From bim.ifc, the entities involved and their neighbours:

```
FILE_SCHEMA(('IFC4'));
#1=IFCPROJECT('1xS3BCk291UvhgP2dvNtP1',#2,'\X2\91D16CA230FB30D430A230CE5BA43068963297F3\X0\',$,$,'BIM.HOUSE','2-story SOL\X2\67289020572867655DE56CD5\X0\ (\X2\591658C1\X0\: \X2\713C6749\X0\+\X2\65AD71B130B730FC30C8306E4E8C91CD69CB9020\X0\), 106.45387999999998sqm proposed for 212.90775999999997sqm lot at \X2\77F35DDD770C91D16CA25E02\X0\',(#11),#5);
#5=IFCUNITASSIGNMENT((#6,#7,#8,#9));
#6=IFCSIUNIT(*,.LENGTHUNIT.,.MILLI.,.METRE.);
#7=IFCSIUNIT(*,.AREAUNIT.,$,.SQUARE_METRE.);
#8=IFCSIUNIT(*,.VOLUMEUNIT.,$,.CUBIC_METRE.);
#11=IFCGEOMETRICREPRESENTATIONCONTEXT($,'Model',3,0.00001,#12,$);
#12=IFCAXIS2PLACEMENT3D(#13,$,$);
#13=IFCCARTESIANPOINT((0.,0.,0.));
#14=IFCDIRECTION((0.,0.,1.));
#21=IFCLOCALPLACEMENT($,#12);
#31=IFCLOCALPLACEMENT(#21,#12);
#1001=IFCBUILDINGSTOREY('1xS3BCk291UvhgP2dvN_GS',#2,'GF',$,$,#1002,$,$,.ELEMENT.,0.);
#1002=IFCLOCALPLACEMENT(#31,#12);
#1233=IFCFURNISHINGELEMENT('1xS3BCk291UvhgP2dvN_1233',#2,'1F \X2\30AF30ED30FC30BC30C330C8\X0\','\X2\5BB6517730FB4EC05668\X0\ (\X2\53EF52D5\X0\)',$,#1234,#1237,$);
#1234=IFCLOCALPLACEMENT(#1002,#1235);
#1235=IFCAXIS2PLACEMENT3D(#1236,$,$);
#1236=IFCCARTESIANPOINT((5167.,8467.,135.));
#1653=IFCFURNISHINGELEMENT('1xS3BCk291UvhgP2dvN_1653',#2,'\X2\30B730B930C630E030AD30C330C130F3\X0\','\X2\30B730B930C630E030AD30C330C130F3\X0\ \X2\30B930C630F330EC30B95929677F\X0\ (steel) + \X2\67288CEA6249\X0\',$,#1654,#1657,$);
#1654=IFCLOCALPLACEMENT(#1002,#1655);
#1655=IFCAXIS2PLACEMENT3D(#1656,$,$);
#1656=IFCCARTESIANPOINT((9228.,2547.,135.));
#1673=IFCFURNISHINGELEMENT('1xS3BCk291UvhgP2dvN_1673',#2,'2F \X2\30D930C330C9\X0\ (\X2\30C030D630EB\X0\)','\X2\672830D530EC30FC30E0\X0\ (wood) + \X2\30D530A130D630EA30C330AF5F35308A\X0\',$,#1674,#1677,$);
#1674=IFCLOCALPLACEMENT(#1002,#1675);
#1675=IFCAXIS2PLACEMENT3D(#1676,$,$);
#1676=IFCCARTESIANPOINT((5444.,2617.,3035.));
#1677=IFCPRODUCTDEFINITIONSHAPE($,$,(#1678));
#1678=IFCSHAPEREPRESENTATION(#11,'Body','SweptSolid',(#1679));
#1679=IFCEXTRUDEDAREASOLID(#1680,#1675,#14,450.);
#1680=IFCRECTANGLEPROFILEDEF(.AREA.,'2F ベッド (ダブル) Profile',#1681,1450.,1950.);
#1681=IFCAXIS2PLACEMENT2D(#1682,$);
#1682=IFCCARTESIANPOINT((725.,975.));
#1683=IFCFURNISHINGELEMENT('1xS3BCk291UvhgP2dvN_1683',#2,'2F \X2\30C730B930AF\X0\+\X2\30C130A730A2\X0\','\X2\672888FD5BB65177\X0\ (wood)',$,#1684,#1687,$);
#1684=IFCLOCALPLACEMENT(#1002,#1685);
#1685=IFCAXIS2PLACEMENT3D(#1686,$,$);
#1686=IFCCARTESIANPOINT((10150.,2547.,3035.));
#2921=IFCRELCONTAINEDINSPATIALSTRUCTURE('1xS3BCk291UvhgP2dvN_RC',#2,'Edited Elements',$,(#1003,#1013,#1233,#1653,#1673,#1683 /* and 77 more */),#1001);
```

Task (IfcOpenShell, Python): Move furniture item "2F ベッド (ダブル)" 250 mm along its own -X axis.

```python
import ifcopenshell
import ifcopenshell.api.geometry
import ifcopenshell.util.placement

model = ifcopenshell.open("bim.ifc")

item = model.by_guid("1xS3BCk291UvhgP2dvN_1673")
matrix = ifcopenshell.util.placement.get_local_placement(item.ObjectPlacement)
matrix[:3, 3] -= matrix[:3, 0] * 250.0
ifcopenshell.api.geometry.edit_object_placement(model, product=item, matrix=matrix, is_si=False)

print(ifcopenshell.util.placement.get_local_placement(item.ObjectPlacement).round(3) + 0.0)

model.write("bim_v2.ifc")
```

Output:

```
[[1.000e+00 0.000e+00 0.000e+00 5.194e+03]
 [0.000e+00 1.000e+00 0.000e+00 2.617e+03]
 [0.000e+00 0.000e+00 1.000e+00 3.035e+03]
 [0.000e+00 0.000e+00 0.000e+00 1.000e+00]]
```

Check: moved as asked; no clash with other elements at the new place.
